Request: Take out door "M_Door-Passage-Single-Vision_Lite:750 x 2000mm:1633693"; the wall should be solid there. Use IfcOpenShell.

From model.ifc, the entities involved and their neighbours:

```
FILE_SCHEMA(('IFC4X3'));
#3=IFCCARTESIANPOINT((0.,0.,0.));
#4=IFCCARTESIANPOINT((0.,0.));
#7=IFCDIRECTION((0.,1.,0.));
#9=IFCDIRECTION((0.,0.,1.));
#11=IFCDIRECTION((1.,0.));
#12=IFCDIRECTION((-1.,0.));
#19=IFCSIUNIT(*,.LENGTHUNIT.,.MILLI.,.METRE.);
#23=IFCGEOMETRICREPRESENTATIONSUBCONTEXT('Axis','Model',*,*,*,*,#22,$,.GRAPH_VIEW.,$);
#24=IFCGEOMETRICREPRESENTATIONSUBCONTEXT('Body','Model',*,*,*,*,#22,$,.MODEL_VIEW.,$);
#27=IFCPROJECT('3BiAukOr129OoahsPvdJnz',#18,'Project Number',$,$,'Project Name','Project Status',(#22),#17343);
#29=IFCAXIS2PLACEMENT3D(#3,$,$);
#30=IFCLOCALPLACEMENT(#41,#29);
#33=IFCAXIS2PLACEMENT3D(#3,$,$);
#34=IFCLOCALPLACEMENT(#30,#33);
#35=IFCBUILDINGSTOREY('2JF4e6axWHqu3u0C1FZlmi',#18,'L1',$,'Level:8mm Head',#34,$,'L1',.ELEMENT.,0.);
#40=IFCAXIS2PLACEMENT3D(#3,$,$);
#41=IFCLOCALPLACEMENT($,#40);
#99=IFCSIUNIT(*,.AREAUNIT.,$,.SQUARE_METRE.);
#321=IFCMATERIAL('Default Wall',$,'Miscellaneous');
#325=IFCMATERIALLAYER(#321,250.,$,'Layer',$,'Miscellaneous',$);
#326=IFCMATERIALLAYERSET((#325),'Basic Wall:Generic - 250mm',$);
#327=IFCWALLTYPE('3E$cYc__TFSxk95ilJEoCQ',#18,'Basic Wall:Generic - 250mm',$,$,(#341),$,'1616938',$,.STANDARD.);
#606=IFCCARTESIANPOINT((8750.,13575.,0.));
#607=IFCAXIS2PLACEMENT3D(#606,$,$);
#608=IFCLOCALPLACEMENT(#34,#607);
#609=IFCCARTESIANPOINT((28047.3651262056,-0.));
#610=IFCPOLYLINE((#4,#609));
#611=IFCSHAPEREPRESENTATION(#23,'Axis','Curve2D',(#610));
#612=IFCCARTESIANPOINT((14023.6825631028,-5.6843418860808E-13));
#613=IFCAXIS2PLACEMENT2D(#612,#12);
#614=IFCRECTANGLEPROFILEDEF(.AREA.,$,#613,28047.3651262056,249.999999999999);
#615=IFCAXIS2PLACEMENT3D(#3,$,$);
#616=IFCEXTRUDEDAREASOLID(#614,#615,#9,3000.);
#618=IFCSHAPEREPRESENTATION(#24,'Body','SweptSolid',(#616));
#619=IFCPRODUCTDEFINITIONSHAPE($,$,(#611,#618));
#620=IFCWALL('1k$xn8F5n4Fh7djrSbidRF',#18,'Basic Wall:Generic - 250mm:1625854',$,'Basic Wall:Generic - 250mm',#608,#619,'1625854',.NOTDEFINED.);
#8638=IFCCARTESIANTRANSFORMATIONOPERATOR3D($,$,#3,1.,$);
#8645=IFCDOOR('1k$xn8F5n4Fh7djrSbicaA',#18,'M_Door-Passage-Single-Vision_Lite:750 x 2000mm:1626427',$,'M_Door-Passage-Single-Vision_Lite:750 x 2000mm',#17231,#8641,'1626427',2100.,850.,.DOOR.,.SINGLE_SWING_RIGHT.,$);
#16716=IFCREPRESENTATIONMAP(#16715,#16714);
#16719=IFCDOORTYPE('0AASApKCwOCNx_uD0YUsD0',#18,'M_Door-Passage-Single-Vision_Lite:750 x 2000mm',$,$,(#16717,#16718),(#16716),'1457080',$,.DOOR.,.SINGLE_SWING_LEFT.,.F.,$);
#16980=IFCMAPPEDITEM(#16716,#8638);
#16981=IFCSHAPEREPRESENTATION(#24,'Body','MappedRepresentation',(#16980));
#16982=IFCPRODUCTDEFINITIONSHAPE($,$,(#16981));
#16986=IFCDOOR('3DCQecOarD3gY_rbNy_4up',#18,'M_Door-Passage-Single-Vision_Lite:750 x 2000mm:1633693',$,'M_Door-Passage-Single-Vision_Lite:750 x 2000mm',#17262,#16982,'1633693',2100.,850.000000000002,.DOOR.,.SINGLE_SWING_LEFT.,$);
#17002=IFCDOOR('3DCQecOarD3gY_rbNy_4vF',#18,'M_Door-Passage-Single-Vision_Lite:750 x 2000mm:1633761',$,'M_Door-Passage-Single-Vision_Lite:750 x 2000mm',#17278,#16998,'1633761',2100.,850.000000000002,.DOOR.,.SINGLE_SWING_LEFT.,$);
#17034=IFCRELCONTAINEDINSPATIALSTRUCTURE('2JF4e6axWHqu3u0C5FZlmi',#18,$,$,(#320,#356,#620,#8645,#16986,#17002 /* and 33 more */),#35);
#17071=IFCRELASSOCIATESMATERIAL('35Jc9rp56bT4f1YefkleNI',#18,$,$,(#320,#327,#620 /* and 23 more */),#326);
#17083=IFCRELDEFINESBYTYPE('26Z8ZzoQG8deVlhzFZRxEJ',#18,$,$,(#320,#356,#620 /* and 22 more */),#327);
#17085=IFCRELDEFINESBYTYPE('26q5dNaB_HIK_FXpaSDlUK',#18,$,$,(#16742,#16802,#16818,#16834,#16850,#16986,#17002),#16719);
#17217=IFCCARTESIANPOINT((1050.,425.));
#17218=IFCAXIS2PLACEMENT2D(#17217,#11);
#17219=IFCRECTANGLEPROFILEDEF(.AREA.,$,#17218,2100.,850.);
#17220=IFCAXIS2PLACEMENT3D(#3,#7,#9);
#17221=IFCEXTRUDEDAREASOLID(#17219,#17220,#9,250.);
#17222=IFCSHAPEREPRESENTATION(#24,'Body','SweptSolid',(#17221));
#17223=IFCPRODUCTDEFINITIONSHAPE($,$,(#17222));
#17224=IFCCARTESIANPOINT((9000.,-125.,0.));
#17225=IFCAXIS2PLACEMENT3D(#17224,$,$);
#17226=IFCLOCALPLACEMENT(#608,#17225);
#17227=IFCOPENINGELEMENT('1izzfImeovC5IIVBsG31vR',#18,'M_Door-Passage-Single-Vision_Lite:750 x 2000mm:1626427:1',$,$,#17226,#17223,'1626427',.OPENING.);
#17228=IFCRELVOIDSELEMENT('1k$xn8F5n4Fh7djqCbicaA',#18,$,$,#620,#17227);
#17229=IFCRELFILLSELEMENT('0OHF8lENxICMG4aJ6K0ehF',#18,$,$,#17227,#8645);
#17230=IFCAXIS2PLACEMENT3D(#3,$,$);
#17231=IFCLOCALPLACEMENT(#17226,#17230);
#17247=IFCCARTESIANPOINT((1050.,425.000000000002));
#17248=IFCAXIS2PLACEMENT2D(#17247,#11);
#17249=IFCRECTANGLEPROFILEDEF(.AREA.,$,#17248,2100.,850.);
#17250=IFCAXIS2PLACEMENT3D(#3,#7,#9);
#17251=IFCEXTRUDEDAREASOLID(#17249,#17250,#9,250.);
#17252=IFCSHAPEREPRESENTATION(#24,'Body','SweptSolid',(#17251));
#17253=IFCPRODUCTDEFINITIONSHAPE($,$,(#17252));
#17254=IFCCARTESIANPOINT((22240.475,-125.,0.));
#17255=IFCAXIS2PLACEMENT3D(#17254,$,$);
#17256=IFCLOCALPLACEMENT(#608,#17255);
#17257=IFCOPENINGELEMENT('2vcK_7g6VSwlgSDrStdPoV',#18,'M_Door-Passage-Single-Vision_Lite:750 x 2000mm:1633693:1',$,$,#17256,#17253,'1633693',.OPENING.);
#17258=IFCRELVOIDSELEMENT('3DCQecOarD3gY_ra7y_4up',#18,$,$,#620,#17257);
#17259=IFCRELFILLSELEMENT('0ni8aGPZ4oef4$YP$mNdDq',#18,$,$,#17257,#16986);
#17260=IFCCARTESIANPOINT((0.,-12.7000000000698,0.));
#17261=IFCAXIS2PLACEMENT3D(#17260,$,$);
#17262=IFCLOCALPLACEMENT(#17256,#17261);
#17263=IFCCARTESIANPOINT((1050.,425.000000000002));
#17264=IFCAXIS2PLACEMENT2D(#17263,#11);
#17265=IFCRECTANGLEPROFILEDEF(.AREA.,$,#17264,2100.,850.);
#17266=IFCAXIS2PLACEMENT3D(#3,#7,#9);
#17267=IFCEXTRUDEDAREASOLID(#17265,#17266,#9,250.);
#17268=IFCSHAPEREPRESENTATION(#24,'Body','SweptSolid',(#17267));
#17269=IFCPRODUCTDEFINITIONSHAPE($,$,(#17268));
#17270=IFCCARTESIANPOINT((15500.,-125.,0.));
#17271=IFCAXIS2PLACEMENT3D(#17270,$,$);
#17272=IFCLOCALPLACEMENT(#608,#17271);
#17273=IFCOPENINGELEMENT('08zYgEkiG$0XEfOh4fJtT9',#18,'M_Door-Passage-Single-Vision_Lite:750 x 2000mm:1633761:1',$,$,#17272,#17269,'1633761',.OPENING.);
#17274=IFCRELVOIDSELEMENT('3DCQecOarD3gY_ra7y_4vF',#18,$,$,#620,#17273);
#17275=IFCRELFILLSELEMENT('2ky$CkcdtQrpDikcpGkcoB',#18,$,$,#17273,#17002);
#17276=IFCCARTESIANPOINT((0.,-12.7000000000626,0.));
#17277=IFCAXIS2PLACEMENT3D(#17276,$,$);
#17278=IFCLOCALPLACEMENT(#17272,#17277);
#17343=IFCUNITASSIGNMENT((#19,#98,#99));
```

```python
import ifcopenshell
import ifcopenshell.api.feature
import ifcopenshell.api.root
import ifcopenshell.geom
import ifcopenshell.util.shape

model = ifcopenshell.open("model.ifc")
settings = ifcopenshell.geom.settings()


def volume(element):
    """Net volume in cubic metres, openings subtracted."""
    shape = ifcopenshell.geom.create_shape(settings, element)
    return ifcopenshell.util.shape.get_volume(shape.geometry)


door = model.by_guid("3DCQecOarD3gY_rbNy_4up")
opening = door.FillsVoids[0].RelatingOpeningElement
wall = opening.VoidsElements[0].RelatingBuildingElement
before = volume(wall)

ifcopenshell.api.root.remove_product(model, product=door)
ifcopenshell.api.feature.remove_feature(model, feature=opening)

after = volume(wall)

print(f"wall volume {before:.3f} -> {after:.3f} m3")

model.write("model_rev.ifc")
```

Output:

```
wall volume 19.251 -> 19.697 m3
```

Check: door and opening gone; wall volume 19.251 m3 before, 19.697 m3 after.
